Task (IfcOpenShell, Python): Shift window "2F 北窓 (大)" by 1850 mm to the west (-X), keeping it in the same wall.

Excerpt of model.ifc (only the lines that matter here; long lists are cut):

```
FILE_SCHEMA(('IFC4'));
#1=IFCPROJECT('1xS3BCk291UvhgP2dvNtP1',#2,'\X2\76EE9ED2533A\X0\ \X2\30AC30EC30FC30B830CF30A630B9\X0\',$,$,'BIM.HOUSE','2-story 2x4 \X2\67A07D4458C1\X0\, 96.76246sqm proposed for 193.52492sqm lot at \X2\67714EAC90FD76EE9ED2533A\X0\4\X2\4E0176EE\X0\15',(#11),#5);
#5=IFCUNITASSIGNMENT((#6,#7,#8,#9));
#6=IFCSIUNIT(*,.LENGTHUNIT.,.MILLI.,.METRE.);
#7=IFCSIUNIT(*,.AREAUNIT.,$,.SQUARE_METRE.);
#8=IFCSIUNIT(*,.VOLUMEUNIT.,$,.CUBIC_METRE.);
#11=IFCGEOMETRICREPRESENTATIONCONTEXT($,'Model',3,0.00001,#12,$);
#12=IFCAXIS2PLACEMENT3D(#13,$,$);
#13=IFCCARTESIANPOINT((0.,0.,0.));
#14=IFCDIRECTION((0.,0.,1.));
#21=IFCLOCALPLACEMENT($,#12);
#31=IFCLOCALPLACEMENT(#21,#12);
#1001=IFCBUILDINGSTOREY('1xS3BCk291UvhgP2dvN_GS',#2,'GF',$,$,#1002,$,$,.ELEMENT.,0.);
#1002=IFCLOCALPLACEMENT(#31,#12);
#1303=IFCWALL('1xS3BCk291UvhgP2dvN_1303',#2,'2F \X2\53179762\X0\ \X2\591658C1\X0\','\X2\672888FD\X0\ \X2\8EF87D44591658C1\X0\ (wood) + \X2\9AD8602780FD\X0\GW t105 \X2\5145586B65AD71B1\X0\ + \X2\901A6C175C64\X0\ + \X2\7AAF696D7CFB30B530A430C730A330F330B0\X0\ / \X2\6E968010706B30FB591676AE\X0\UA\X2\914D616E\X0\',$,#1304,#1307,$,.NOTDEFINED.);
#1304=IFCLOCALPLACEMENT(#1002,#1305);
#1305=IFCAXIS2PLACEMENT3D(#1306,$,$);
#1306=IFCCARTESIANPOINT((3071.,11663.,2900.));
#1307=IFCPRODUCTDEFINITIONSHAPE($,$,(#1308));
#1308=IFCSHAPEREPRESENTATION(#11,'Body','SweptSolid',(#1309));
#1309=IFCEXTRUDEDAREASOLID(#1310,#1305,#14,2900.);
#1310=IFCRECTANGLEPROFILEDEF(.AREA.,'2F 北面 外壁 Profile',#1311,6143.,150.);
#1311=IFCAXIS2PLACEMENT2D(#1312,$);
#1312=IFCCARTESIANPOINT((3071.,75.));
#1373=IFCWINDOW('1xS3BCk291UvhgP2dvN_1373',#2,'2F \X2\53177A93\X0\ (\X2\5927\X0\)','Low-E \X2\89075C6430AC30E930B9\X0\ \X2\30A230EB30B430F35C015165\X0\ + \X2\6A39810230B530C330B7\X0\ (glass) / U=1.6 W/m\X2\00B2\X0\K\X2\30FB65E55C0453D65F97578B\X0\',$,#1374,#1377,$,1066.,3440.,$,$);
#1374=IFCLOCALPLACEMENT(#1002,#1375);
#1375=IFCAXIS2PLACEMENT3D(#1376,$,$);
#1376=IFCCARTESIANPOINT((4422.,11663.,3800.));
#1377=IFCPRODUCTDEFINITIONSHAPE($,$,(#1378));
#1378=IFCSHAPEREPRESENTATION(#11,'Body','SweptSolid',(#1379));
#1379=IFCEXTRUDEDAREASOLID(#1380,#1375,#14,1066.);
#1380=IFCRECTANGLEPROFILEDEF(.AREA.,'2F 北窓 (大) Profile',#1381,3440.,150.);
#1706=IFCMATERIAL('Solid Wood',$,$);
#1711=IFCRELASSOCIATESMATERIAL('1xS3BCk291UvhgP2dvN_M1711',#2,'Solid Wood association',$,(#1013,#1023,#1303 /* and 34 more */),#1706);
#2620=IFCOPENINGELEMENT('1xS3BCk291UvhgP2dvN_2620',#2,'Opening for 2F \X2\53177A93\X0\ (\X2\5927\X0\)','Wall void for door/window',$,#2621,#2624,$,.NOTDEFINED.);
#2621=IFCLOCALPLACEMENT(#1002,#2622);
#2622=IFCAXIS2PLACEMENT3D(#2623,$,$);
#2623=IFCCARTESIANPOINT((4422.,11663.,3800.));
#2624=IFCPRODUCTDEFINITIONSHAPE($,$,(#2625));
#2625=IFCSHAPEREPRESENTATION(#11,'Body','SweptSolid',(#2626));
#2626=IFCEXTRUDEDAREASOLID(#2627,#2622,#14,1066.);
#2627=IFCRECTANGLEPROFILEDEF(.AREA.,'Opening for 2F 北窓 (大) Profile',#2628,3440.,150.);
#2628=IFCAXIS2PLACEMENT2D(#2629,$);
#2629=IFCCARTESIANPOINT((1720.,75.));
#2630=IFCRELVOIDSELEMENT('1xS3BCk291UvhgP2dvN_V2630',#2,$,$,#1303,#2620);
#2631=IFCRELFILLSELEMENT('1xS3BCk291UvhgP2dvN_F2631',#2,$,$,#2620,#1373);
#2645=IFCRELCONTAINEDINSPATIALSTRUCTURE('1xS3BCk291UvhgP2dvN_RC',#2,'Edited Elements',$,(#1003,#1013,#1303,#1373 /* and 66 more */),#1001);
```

```python
import ifcopenshell
import ifcopenshell.api.geometry
import ifcopenshell.util.placement
import ifcopenshell.util.unit

model = ifcopenshell.open("model.ifc")
unit_scale = ifcopenshell.util.unit.calculate_unit_scale(model)

window = model.by_id(1373)
opening = window.FillsVoids[0].RelatingOpeningElement
wall = opening.VoidsElements[0].RelatingBuildingElement

wall_matrix = ifcopenshell.util.placement.get_local_placement(wall.ObjectPlacement)
shift = wall_matrix[:3, 0] * -1.85 / unit_scale
before = ifcopenshell.util.placement.get_local_placement(window.ObjectPlacement)[:3, 3].copy()

# The window is not placed relative to its opening, so move both.
for product in (opening, window):
    matrix = ifcopenshell.util.placement.get_local_placement(product.ObjectPlacement)
    matrix[:3, 3] += shift
    ifcopenshell.api.geometry.edit_object_placement(model, product=product, matrix=matrix, is_si=False)

after = ifcopenshell.util.placement.get_local_placement(window.ObjectPlacement)[:3, 3]
print("window moved by", (after - before).round(3) + 0.0)

model.write("model-out.ifc")
```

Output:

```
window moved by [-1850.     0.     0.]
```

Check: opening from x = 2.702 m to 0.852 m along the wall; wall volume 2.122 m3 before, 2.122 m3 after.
